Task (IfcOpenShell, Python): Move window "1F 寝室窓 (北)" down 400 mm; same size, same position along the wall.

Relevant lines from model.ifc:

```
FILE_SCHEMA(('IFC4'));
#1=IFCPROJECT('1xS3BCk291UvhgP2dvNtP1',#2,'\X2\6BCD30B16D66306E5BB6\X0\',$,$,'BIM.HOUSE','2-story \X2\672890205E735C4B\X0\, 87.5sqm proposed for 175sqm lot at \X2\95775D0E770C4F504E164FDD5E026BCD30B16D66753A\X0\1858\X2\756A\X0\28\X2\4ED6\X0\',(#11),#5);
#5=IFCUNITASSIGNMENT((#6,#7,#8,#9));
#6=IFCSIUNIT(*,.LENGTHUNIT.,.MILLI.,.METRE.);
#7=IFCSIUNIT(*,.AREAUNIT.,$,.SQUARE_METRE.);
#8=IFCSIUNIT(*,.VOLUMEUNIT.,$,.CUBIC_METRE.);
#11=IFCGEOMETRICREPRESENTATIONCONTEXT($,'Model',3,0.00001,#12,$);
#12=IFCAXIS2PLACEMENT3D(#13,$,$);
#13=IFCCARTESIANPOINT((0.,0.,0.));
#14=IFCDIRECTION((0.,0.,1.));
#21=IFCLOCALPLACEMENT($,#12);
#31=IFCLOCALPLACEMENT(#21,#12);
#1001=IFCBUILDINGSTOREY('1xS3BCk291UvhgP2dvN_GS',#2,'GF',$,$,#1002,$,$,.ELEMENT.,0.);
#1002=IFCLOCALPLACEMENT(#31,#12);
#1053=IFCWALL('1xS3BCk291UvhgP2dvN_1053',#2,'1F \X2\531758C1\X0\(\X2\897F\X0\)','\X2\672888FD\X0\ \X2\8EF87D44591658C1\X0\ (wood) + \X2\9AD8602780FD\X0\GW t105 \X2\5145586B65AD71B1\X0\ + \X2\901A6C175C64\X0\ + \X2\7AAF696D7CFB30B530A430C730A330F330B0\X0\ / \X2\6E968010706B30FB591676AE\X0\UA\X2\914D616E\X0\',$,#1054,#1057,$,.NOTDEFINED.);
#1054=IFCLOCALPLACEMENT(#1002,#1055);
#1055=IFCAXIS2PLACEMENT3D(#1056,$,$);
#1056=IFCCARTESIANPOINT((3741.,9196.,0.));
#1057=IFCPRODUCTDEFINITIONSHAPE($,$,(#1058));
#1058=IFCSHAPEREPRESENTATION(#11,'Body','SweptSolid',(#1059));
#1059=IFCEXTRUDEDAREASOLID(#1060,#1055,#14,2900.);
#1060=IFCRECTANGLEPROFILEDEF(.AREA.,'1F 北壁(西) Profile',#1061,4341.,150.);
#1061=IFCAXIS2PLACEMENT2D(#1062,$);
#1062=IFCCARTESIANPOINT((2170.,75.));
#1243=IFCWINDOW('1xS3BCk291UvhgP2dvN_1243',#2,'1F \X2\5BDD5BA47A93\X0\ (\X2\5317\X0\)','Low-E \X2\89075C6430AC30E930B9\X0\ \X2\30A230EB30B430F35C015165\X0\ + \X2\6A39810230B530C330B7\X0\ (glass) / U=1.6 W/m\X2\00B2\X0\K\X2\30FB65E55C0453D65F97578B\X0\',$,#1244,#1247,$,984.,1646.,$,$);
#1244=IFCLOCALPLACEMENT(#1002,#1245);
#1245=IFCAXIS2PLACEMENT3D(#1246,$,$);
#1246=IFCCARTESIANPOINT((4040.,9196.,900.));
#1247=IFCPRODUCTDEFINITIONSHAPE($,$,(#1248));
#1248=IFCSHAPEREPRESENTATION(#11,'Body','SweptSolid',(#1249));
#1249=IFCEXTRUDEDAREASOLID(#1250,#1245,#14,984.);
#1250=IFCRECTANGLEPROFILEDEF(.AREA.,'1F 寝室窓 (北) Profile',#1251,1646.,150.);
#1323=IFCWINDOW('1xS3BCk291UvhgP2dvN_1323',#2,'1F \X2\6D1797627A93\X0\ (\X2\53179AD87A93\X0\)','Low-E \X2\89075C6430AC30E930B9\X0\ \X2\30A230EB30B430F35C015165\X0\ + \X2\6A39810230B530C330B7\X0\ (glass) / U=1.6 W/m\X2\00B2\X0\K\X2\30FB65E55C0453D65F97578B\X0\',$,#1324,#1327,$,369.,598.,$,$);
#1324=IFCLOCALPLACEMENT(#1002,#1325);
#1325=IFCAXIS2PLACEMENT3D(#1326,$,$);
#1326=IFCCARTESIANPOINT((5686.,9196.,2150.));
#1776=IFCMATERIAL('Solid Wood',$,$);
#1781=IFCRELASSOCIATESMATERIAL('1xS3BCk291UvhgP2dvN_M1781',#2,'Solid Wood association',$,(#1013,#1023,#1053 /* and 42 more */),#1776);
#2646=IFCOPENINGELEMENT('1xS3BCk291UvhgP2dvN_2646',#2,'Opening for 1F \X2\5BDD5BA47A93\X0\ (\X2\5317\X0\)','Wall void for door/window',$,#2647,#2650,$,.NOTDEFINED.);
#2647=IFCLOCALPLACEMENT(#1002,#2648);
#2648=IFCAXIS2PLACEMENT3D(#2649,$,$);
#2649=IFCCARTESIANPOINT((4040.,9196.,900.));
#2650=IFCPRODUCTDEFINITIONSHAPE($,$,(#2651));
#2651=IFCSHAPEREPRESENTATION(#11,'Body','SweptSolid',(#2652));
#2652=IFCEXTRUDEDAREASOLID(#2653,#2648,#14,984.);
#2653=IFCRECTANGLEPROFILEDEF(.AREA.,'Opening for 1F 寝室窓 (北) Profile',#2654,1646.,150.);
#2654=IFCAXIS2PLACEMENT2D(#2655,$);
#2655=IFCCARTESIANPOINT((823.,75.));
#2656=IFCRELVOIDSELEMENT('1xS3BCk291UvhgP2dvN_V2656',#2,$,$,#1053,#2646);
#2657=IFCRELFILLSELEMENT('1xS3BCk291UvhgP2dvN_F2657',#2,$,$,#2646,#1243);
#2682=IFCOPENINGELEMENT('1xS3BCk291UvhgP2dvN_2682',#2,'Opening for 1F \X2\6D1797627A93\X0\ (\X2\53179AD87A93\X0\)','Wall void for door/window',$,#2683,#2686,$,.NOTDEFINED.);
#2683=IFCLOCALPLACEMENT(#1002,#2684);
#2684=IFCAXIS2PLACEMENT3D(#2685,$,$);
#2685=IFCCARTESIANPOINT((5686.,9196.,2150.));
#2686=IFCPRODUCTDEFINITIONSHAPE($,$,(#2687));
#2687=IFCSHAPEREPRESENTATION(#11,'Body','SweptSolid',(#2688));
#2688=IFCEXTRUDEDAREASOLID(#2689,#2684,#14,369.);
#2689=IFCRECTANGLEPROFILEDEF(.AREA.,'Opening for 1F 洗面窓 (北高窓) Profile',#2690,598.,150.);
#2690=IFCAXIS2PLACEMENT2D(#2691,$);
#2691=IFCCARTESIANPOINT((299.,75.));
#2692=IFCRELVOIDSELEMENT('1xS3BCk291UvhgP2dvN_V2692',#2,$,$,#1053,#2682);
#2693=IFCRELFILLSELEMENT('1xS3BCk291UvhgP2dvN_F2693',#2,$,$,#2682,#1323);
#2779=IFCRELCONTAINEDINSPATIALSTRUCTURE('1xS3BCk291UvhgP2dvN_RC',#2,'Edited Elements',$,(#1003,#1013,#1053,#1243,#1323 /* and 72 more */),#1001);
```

```python
import numpy as np
import ifcopenshell
import ifcopenshell.api.geometry
import ifcopenshell.util.placement
import ifcopenshell.util.unit

model = ifcopenshell.open("model.ifc")
unit_scale = ifcopenshell.util.unit.calculate_unit_scale(model)

window = model.by_guid("1xS3BCk291UvhgP2dvN_1243")
opening = window.FillsVoids[0].RelatingOpeningElement
dz = -400.0

shift = np.array([0.0, 0.0, dz])
# The window is not placed relative to its opening, so move both.
for product in (opening, window):
    matrix = ifcopenshell.util.placement.get_local_placement(product.ObjectPlacement)
    matrix[:3, 3] += shift
    ifcopenshell.api.geometry.edit_object_placement(model, product=product, matrix=matrix, is_si=False)

print(f"moved by {dz * unit_scale:+.3f} m")

model.write("model_v2.ifc")
```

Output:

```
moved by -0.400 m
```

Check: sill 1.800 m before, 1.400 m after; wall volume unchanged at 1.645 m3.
